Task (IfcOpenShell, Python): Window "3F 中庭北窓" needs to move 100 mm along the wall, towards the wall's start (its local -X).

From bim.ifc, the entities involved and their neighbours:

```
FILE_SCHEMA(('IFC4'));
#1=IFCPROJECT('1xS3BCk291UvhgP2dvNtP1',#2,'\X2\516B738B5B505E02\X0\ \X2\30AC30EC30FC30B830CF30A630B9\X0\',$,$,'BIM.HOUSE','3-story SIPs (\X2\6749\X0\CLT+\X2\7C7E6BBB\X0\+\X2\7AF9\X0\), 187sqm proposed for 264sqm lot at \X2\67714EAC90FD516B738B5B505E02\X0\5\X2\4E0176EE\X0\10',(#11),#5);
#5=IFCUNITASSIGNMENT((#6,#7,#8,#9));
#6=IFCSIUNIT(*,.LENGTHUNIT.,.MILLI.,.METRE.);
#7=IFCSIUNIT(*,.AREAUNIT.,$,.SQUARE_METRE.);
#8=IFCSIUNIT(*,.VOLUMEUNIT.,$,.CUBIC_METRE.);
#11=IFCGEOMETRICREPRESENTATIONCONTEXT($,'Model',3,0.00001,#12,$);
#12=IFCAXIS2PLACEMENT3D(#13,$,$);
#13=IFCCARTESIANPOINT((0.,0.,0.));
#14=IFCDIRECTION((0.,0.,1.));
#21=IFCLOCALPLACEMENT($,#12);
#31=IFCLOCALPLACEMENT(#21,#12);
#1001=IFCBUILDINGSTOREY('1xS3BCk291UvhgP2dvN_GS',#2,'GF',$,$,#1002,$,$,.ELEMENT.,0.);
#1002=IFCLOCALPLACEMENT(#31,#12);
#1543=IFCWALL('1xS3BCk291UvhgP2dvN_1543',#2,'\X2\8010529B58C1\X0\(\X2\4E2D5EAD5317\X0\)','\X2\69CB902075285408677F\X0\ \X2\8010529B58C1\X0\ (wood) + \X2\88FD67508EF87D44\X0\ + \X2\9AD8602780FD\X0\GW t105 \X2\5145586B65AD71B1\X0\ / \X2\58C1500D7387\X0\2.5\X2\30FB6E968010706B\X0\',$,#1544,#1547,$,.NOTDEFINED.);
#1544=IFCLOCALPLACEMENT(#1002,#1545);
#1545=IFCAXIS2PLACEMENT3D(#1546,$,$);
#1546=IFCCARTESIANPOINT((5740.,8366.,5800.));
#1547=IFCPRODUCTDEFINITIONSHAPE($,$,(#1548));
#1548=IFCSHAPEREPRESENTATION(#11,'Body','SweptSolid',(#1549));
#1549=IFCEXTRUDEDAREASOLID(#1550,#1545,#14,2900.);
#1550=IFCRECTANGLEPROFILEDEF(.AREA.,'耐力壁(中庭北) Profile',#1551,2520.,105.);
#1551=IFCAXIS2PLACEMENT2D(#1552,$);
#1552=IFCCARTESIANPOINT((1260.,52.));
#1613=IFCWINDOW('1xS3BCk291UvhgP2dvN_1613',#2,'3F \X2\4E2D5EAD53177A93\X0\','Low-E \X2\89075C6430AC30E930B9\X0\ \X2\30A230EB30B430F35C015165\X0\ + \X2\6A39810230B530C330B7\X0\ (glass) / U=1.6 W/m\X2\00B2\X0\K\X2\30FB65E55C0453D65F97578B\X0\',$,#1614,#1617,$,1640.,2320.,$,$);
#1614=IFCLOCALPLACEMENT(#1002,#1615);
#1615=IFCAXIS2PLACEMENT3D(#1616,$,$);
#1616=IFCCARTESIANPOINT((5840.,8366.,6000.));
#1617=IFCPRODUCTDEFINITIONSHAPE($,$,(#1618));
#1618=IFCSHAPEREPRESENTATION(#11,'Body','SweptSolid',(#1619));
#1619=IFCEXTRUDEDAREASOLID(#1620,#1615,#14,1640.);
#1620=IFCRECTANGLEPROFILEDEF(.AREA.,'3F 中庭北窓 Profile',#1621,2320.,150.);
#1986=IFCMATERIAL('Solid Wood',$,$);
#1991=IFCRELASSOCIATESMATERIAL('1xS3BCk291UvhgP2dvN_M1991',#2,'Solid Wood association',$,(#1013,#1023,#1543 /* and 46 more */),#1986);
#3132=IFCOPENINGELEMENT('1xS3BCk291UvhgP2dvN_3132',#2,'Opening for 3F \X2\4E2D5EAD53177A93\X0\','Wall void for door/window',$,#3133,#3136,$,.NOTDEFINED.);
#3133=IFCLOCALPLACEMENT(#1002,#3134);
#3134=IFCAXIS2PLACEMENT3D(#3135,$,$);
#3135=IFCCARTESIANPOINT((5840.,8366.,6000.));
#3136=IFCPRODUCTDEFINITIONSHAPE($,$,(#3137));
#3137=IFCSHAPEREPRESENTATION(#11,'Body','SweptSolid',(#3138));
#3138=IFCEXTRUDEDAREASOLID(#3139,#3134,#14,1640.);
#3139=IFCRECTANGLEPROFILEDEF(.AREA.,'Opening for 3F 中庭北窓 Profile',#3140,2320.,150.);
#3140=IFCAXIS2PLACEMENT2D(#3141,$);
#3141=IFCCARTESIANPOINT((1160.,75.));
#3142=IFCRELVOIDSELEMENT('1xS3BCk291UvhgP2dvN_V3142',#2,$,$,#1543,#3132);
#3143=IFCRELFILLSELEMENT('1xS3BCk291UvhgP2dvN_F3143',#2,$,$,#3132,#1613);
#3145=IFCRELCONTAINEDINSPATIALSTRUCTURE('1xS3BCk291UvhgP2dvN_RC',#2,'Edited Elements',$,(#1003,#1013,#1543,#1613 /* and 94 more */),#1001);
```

```python
import ifcopenshell
import ifcopenshell.api.geometry
import ifcopenshell.util.placement

model = ifcopenshell.open("bim.ifc")

window = model.by_guid("1xS3BCk291UvhgP2dvN_1613")
opening = window.FillsVoids[0].RelatingOpeningElement
wall = opening.VoidsElements[0].RelatingBuildingElement

wall_matrix = ifcopenshell.util.placement.get_local_placement(wall.ObjectPlacement)
shift = wall_matrix[:3, 0] * -100.0
before = ifcopenshell.util.placement.get_local_placement(window.ObjectPlacement)[:3, 3].copy()

# The window is not placed relative to its opening, so move both.
for product in (opening, window):
    matrix = ifcopenshell.util.placement.get_local_placement(product.ObjectPlacement)
    matrix[:3, 3] += shift
    ifcopenshell.api.geometry.edit_object_placement(model, product=product, matrix=matrix, is_si=False)

after = ifcopenshell.util.placement.get_local_placement(window.ObjectPlacement)[:3, 3]
print("window moved by", (after - before).round(3) + 0.0)

model.write("bim_updated.ifc")
```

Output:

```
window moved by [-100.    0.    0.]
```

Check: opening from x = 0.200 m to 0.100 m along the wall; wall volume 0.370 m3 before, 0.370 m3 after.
